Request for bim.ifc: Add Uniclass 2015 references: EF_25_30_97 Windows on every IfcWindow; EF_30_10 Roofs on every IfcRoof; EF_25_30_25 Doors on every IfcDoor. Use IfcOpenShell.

First a look at what the model holds.

```python
import ifcopenshell

model = ifcopenshell.open("bim.ifc")
print(model.schema)
print("classifications:", [c.Name for c in model.by_type("IfcClassification")])
for ifc_class in ("IfcDoor", "IfcRoof", "IfcStair", "IfcWall", "IfcWindow"):
    print(ifc_class, len(model.by_type(ifc_class)))
```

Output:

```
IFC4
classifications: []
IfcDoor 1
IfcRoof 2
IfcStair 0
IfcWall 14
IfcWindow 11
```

```python
import ifcopenshell
import ifcopenshell.api.classification

model = ifcopenshell.open("bim.ifc")

system = ifcopenshell.api.classification.add_classification(model, classification="Uniclass 2015")

codes = {
    "IfcWindow": ("EF_25_30_97", "Windows"),
    "IfcRoof": ("EF_30_10", "Roofs"),
    "IfcDoor": ("EF_25_30_25", "Doors"),
}
for ifc_class, (code, name) in codes.items():
    products = model.by_type(ifc_class)
    ifcopenshell.api.classification.add_reference(
        model, products=products, classification=system, identification=code, name=name
    )
    print(code, len(products))

model.write("bim_edited.ifc")
```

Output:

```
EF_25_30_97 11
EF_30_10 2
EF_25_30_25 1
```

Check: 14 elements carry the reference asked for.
